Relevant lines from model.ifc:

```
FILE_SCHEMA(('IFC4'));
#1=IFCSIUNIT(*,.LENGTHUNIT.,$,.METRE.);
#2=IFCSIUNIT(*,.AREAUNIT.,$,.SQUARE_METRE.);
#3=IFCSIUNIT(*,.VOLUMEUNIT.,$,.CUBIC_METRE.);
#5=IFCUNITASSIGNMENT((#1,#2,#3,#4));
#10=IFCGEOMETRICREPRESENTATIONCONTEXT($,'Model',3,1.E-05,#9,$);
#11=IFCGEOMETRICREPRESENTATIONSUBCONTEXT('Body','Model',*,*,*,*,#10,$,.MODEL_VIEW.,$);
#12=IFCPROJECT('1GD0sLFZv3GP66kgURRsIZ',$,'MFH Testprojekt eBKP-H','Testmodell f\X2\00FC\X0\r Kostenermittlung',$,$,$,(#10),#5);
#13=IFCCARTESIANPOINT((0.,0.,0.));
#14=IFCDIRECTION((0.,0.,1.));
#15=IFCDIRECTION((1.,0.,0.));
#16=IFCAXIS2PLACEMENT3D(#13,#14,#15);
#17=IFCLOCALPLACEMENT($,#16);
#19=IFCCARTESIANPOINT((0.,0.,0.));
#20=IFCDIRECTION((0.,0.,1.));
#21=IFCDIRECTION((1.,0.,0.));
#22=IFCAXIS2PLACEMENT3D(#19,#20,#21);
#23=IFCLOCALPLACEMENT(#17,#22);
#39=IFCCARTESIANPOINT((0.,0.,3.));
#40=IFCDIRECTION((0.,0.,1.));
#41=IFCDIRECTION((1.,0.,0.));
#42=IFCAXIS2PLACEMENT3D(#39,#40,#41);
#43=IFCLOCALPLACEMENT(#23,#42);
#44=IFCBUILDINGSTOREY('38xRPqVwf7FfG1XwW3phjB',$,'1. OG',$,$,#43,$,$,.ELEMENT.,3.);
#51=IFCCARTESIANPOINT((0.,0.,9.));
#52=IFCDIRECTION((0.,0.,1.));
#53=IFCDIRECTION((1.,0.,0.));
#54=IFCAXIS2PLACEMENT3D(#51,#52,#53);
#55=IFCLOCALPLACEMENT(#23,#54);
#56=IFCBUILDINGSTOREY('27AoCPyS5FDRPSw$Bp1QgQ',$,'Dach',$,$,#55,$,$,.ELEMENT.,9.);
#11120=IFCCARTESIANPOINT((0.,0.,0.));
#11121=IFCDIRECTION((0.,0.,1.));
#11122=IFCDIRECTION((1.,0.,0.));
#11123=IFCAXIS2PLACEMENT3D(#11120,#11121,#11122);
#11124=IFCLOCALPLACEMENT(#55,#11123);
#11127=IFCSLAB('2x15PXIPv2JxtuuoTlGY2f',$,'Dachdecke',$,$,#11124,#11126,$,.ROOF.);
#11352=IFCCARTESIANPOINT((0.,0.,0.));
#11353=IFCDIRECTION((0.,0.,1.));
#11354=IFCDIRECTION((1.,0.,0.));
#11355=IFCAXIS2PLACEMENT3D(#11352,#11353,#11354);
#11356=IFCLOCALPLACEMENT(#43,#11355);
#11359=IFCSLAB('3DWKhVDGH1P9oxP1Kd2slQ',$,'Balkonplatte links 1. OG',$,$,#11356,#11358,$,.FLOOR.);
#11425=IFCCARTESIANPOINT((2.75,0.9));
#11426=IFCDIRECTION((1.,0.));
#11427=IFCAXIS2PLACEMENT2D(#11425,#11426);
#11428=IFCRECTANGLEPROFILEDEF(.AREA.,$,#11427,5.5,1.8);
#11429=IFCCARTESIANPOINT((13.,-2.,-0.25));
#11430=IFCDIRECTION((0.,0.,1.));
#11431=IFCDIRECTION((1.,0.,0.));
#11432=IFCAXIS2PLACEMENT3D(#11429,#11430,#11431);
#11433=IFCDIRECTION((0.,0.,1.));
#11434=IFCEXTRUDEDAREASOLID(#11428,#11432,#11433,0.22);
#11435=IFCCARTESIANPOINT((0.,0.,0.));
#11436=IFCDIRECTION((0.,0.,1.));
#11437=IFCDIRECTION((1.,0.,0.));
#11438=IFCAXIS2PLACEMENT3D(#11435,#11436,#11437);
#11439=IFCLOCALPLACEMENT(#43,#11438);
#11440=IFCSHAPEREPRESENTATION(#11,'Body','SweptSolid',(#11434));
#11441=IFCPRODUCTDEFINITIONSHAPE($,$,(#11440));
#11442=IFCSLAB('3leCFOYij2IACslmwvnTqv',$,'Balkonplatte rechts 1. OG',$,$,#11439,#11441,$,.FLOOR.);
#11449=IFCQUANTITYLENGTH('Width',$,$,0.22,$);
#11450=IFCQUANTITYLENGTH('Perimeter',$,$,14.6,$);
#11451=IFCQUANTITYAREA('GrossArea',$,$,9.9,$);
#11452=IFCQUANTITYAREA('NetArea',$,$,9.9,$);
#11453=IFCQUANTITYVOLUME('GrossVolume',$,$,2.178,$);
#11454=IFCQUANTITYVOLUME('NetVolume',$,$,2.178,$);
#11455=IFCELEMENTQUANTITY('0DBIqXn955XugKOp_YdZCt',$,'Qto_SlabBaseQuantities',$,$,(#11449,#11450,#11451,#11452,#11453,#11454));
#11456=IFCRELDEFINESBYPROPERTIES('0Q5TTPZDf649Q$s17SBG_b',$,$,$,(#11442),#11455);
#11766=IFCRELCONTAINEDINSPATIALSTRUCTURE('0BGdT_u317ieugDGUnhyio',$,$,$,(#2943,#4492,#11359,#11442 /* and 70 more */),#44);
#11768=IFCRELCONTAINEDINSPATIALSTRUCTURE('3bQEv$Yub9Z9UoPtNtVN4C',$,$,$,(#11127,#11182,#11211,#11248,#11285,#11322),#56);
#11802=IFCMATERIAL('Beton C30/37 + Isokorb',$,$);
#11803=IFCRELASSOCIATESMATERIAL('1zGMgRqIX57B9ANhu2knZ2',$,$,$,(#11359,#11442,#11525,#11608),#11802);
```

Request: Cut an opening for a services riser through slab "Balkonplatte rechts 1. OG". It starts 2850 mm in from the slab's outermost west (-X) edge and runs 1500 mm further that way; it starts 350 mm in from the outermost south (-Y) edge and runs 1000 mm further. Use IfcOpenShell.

```python
import numpy as np
import ifcopenshell
import ifcopenshell.api.feature
import ifcopenshell.api.geometry
import ifcopenshell.api.pset
import ifcopenshell.api.root
import ifcopenshell.geom
import ifcopenshell.util.element
import ifcopenshell.util.placement
import ifcopenshell.util.representation
import ifcopenshell.util.shape
import ifcopenshell.util.unit

model = ifcopenshell.open("model.ifc")
unit_scale = ifcopenshell.util.unit.calculate_unit_scale(model)
area_scale = ifcopenshell.util.unit.calculate_unit_scale(model, "AREAUNIT")
volume_scale = ifcopenshell.util.unit.calculate_unit_scale(model, "VOLUMEUNIT")
settings = ifcopenshell.geom.settings()


def volume(element):
    """Net volume in cubic metres, openings subtracted."""
    shape = ifcopenshell.geom.create_shape(settings, element)
    return ifcopenshell.util.shape.get_volume(shape.geometry)


slab = model.by_guid("3leCFOYij2IACslmwvnTqv")
before = volume(slab)

# Extent in the slab's own axes, in metres. The edges named are its -X and -Y sides.
slab_shape = ifcopenshell.geom.create_shape(settings, slab)
vertices = ifcopenshell.util.shape.get_vertices(slab_shape.geometry)
x_min, y_min, bottom = vertices.min(axis=0)
top = vertices[:, 2].max()

opening = ifcopenshell.api.root.create_entity(model, ifc_class="IfcOpeningElement", name="Services riser opening", predefined_type="OPENING")
context = ifcopenshell.util.representation.get_context(model, "Model", "Body", "MODEL_VIEW")
width, depth = 1.5, 1
outline = [(0.0, 0.0), (width, 0.0), (width, depth), (0.0, depth), (0.0, 0.0)]
# Overshoot both faces by 50 mm so the cut is clean.
shape = ifcopenshell.api.geometry.add_slab_representation(
    model, context=context, depth=top - bottom + 0.1, polyline=outline
)
ifcopenshell.api.geometry.assign_representation(model, product=opening, representation=shape)

matrix = ifcopenshell.util.placement.get_local_placement(slab.ObjectPlacement)
matrix[:, 3] = matrix @ np.append(np.array([x_min + 2.85, y_min + 0.35, bottom - 0.05]) / unit_scale, 1.0)
ifcopenshell.api.geometry.edit_object_placement(model, product=opening, matrix=matrix, is_si=False)
ifcopenshell.api.feature.add_feature(model, feature=opening, element=slab)

after = volume(slab)

# Update the slab's stored quantities.
qto = model.by_id(ifcopenshell.util.element.get_pset(slab, "Qto_SlabBaseQuantities", should_inherit=False)["id"])
ifcopenshell.api.pset.edit_qto(model, qto=qto, properties={
    "NetArea": after / (top - bottom) / area_scale,
    "NetVolume": after / volume_scale,
})

print(f"slab volume {before:.3f} -> {after:.3f} m3")

model.write("model-out.ifc")
```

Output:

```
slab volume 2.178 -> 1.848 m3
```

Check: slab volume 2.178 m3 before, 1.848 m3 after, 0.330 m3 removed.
